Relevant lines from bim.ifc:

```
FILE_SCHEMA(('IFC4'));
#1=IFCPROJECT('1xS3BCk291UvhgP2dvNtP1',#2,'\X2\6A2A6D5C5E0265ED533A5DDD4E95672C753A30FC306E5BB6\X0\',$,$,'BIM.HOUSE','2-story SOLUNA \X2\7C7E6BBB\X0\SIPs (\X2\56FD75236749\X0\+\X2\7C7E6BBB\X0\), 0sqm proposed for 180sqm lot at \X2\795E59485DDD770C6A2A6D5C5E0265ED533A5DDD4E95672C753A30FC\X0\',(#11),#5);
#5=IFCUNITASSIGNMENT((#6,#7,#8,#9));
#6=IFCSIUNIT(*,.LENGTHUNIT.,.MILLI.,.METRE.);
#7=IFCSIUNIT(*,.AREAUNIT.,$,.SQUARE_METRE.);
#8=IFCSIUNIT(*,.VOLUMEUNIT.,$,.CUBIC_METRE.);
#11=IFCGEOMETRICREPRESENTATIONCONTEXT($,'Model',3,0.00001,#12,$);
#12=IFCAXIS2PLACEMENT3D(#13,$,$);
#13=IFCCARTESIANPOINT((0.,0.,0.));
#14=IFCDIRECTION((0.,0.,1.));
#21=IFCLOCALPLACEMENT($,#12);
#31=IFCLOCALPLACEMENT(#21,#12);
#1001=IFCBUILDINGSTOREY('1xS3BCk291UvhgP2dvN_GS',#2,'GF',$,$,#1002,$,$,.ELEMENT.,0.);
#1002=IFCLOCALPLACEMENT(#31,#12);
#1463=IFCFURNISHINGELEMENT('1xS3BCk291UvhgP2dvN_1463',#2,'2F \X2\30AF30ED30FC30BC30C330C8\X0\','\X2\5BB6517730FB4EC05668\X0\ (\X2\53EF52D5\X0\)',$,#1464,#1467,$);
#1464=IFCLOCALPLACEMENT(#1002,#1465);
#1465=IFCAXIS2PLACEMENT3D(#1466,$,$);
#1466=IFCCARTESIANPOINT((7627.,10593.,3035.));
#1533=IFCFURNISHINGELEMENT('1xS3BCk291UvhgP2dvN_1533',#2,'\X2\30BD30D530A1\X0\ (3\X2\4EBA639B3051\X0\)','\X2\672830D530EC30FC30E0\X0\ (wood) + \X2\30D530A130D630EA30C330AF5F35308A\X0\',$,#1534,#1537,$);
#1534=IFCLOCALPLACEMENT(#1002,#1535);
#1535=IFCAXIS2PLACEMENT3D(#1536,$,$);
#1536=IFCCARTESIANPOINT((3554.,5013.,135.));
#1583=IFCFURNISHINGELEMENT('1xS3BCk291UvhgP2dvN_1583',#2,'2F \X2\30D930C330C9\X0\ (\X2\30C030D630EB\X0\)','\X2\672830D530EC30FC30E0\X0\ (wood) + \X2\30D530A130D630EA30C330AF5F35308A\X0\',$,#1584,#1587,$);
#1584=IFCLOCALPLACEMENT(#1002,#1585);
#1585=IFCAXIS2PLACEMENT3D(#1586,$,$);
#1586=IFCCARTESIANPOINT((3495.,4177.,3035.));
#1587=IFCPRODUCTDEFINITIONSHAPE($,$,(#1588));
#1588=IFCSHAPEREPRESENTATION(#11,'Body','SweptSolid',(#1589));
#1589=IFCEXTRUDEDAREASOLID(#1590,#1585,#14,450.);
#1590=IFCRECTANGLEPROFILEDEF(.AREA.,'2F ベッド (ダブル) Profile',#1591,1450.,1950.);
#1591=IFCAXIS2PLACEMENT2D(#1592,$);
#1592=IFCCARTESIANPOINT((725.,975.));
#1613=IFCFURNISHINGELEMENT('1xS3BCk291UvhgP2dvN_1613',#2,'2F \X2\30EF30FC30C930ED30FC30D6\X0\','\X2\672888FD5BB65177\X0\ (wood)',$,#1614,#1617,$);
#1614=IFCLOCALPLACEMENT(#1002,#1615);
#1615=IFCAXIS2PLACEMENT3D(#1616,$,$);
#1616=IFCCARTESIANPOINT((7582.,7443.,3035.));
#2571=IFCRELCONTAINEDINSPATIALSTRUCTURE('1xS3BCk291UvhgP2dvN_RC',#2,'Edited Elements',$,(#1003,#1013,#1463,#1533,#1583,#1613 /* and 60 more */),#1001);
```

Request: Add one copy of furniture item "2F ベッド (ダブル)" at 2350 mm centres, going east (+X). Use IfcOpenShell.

```python
import numpy as np
import ifcopenshell
import ifcopenshell.api.geometry
import ifcopenshell.api.root
import ifcopenshell.util.element
import ifcopenshell.util.placement
import ifcopenshell.util.unit

model = ifcopenshell.open("bim.ifc")
unit_scale = ifcopenshell.util.unit.calculate_unit_scale(model)


def reuse_history(source, copy):
    """copy_class also copies each property set's owner history, people and application; keep the originals."""
    for rel in copy.IsDefinedBy:
        if rel.is_a("IfcRelDefinesByProperties") and (history := rel.RelatingPropertyDefinition.OwnerHistory):
            rel.RelatingPropertyDefinition.OwnerHistory = source.OwnerHistory
            ifcopenshell.util.element.remove_deep2(model, history)


source = model.by_guid("1xS3BCk291UvhgP2dvN_1583")
base = ifcopenshell.util.placement.get_local_placement(source.ObjectPlacement)
step = np.array([1.0, 0.0, 0.0]) * 2.35 / unit_scale

for i in range(1, 2):
    copy = ifcopenshell.api.root.copy_class(model, product=source)
    copy.Representation = ifcopenshell.util.element.copy_deep(
        model, source.Representation, exclude=["IfcGeometricRepresentationContext", "IfcRepresentationMap"]
    )
    reuse_history(source, copy)
    matrix = base.copy()
    matrix[:3, 3] += i * step
    print("added at", matrix[:3, 3].round(3) + 0.0)
    ifcopenshell.api.geometry.edit_object_placement(model, product=copy, matrix=matrix, is_si=False)

model.write("bim_rev.ifc")
```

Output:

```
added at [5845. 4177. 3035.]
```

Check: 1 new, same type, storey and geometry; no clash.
